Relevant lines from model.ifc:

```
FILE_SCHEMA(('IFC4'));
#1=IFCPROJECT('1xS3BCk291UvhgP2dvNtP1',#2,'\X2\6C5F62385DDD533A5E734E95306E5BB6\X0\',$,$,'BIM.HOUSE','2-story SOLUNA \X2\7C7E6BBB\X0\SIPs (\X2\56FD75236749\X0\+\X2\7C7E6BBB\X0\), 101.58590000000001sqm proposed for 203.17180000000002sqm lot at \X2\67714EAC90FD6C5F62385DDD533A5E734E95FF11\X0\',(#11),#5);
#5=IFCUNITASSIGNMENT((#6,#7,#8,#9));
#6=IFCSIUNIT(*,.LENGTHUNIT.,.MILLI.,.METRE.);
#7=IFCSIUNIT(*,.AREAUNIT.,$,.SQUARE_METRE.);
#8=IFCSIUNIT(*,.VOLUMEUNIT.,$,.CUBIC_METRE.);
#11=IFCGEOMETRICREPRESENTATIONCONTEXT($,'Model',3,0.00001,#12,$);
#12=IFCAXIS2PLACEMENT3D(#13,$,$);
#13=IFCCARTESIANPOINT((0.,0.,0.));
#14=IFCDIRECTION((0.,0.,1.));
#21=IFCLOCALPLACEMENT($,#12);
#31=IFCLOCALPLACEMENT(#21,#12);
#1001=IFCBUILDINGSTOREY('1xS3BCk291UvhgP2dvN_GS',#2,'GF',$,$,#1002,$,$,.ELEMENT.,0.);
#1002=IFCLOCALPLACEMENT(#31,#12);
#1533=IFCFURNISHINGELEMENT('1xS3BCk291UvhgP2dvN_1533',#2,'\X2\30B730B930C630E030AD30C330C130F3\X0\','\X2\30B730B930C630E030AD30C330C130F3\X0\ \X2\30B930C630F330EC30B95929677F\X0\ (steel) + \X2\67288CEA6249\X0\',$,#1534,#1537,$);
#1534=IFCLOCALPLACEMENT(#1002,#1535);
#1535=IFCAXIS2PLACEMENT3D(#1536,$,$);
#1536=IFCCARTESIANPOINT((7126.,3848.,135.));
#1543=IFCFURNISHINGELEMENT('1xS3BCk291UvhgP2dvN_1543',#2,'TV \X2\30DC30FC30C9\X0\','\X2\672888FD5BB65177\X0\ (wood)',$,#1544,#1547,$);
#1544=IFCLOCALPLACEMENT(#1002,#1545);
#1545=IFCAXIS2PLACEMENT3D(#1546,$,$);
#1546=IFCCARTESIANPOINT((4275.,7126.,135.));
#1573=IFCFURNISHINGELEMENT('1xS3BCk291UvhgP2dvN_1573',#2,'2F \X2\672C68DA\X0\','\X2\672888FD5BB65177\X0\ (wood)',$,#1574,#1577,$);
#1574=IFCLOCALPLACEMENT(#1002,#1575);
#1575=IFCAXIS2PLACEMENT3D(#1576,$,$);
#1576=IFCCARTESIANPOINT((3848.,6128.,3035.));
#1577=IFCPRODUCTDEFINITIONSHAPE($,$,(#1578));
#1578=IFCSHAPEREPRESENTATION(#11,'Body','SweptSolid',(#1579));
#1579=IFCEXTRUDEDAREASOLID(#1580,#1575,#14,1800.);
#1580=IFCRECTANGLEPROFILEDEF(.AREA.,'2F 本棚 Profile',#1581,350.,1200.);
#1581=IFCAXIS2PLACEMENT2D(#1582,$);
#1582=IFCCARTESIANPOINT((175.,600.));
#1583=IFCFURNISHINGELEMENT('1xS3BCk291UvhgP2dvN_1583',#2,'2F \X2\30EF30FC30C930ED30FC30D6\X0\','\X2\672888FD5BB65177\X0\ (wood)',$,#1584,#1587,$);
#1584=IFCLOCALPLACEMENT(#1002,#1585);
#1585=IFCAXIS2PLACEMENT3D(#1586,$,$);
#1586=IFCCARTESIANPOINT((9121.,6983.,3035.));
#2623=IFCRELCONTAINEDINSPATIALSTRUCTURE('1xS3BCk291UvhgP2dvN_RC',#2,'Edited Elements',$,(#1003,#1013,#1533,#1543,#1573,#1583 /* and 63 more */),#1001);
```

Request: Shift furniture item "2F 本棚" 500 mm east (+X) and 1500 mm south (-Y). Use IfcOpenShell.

```python
import ifcopenshell
import ifcopenshell.api.geometry
import ifcopenshell.util.placement
import ifcopenshell.util.unit

model = ifcopenshell.open("model.ifc")
unit_scale = ifcopenshell.util.unit.calculate_unit_scale(model)

item = model.by_guid("1xS3BCk291UvhgP2dvN_1573")
matrix = ifcopenshell.util.placement.get_local_placement(item.ObjectPlacement)
matrix[0, 3] += 0.5 / unit_scale
matrix[1, 3] -= 1.5 / unit_scale
ifcopenshell.api.geometry.edit_object_placement(model, product=item, matrix=matrix, is_si=False)

print(ifcopenshell.util.placement.get_local_placement(item.ObjectPlacement).round(3) + 0.0)

model.write("model_updated.ifc")
```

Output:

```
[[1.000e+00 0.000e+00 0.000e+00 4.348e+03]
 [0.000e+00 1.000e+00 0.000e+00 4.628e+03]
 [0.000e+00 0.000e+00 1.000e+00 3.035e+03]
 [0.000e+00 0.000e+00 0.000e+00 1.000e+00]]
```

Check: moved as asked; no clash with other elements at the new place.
